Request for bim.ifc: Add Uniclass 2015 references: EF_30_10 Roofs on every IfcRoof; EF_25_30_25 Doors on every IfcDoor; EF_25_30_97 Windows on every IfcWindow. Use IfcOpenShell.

First a look at what the model holds.

```python
import ifcopenshell

model = ifcopenshell.open("bim.ifc")
print(model.schema)
print("classifications:", [c.Name for c in model.by_type("IfcClassification")])
for ifc_class in ("IfcDoor", "IfcRoof", "IfcStair", "IfcWall", "IfcWindow"):
    print(ifc_class, len(model.by_type(ifc_class)))
```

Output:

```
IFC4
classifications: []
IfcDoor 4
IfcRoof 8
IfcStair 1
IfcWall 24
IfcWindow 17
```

```python
import ifcopenshell
import ifcopenshell.api.classification

model = ifcopenshell.open("bim.ifc")

system = ifcopenshell.api.classification.add_classification(model, classification="Uniclass 2015")

codes = {
    "IfcRoof": ("EF_30_10", "Roofs"),
    "IfcDoor": ("EF_25_30_25", "Doors"),
    "IfcWindow": ("EF_25_30_97", "Windows"),
}
for ifc_class, (code, name) in codes.items():
    products = model.by_type(ifc_class)
    ifcopenshell.api.classification.add_reference(
        model, products=products, classification=system, identification=code, name=name
    )
    print(code, len(products))

model.write("bim-out.ifc")
```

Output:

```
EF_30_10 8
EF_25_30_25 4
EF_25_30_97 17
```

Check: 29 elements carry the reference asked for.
